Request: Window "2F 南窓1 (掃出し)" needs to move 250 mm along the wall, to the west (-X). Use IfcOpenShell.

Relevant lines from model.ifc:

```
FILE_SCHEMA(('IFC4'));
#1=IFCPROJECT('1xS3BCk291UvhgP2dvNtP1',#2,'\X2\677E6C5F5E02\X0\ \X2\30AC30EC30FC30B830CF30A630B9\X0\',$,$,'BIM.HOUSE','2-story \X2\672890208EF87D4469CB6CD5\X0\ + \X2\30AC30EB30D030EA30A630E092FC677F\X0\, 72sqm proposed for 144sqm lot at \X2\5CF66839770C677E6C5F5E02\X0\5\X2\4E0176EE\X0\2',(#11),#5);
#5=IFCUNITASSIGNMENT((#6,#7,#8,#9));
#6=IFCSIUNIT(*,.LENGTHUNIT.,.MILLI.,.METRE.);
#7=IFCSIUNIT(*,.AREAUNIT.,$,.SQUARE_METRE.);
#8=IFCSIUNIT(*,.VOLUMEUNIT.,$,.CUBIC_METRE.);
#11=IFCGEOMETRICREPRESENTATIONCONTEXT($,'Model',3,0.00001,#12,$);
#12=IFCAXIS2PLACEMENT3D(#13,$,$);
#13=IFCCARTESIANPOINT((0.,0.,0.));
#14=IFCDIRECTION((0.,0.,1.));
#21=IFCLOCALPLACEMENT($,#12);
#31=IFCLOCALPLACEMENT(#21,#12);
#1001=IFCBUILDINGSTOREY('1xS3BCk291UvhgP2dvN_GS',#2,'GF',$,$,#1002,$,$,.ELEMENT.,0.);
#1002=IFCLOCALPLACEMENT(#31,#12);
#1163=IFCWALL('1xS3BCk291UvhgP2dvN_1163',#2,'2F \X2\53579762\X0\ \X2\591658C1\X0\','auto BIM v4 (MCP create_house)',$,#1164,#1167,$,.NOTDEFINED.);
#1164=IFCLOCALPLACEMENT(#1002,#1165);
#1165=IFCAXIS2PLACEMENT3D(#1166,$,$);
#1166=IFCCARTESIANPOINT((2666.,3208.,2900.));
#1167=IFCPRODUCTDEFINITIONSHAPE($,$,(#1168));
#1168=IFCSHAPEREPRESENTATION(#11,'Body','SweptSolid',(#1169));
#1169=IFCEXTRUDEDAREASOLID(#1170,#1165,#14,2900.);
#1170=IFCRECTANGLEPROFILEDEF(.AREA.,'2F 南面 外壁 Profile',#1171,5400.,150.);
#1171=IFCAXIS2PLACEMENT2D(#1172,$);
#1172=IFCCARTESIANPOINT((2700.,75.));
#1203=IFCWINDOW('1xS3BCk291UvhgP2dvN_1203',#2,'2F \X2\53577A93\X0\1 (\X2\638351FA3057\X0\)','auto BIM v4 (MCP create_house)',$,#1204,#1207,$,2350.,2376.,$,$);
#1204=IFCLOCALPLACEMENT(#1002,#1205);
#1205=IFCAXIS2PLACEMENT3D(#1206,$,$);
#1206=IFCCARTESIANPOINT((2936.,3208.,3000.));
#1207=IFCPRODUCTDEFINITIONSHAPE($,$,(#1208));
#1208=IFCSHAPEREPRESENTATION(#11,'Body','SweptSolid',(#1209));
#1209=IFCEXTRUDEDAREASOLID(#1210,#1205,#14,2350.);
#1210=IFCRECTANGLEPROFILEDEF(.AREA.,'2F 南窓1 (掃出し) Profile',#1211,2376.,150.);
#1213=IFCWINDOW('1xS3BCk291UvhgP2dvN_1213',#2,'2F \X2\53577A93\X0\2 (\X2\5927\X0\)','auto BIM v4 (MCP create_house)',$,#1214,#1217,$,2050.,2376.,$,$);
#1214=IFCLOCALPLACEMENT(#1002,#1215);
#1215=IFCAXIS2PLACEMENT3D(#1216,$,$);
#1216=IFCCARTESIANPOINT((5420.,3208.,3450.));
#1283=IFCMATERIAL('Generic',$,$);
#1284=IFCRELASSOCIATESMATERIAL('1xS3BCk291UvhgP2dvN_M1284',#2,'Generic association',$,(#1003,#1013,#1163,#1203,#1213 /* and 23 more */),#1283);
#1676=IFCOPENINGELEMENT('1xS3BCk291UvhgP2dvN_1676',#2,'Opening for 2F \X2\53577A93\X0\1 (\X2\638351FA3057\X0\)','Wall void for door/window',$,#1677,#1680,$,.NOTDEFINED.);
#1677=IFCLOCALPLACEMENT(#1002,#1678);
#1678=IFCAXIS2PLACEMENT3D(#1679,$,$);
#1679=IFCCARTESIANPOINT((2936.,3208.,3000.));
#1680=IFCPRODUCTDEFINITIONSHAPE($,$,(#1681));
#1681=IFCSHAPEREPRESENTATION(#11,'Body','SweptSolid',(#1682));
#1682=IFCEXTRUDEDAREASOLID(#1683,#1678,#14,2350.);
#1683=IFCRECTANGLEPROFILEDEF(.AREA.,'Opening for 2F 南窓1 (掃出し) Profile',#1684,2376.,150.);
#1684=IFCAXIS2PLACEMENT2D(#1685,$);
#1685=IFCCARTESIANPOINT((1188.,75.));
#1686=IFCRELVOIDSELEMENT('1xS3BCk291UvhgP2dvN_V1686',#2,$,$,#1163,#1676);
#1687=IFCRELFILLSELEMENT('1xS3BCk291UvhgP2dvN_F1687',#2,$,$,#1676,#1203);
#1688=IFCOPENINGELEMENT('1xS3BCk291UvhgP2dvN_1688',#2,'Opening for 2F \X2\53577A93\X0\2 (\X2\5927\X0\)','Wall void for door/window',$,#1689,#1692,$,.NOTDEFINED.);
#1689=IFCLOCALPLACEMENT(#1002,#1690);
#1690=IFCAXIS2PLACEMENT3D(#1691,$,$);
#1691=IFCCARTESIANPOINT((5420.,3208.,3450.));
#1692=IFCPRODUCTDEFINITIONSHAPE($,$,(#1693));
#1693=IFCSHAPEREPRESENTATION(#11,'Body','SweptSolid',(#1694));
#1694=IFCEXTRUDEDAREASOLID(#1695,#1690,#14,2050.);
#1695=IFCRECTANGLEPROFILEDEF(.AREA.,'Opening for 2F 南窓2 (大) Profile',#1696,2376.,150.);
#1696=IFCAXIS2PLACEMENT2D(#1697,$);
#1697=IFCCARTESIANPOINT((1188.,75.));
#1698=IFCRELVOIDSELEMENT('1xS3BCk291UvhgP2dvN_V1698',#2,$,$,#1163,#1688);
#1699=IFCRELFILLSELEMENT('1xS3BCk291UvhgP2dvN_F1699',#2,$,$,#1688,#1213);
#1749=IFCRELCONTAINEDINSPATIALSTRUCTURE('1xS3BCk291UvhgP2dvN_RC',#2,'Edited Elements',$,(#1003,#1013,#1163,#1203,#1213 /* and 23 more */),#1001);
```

```python
import ifcopenshell
import ifcopenshell.api.geometry
import ifcopenshell.util.placement
import ifcopenshell.util.unit

model = ifcopenshell.open("model.ifc")
unit_scale = ifcopenshell.util.unit.calculate_unit_scale(model)

window = model.by_guid("1xS3BCk291UvhgP2dvN_1203")
opening = window.FillsVoids[0].RelatingOpeningElement
wall = opening.VoidsElements[0].RelatingBuildingElement

wall_matrix = ifcopenshell.util.placement.get_local_placement(wall.ObjectPlacement)
shift = wall_matrix[:3, 0] * -0.25 / unit_scale
before = ifcopenshell.util.placement.get_local_placement(window.ObjectPlacement)[:3, 3].copy()

# The window is not placed relative to its opening, so move both.
for product in (opening, window):
    matrix = ifcopenshell.util.placement.get_local_placement(product.ObjectPlacement)
    matrix[:3, 3] += shift
    ifcopenshell.api.geometry.edit_object_placement(model, product=product, matrix=matrix, is_si=False)

after = ifcopenshell.util.placement.get_local_placement(window.ObjectPlacement)[:3, 3]
print("window moved by", (after - before).round(3) + 0.0)

model.write("model-out.ifc")
```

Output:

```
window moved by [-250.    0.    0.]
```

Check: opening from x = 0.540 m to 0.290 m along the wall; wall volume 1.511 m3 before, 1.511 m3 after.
